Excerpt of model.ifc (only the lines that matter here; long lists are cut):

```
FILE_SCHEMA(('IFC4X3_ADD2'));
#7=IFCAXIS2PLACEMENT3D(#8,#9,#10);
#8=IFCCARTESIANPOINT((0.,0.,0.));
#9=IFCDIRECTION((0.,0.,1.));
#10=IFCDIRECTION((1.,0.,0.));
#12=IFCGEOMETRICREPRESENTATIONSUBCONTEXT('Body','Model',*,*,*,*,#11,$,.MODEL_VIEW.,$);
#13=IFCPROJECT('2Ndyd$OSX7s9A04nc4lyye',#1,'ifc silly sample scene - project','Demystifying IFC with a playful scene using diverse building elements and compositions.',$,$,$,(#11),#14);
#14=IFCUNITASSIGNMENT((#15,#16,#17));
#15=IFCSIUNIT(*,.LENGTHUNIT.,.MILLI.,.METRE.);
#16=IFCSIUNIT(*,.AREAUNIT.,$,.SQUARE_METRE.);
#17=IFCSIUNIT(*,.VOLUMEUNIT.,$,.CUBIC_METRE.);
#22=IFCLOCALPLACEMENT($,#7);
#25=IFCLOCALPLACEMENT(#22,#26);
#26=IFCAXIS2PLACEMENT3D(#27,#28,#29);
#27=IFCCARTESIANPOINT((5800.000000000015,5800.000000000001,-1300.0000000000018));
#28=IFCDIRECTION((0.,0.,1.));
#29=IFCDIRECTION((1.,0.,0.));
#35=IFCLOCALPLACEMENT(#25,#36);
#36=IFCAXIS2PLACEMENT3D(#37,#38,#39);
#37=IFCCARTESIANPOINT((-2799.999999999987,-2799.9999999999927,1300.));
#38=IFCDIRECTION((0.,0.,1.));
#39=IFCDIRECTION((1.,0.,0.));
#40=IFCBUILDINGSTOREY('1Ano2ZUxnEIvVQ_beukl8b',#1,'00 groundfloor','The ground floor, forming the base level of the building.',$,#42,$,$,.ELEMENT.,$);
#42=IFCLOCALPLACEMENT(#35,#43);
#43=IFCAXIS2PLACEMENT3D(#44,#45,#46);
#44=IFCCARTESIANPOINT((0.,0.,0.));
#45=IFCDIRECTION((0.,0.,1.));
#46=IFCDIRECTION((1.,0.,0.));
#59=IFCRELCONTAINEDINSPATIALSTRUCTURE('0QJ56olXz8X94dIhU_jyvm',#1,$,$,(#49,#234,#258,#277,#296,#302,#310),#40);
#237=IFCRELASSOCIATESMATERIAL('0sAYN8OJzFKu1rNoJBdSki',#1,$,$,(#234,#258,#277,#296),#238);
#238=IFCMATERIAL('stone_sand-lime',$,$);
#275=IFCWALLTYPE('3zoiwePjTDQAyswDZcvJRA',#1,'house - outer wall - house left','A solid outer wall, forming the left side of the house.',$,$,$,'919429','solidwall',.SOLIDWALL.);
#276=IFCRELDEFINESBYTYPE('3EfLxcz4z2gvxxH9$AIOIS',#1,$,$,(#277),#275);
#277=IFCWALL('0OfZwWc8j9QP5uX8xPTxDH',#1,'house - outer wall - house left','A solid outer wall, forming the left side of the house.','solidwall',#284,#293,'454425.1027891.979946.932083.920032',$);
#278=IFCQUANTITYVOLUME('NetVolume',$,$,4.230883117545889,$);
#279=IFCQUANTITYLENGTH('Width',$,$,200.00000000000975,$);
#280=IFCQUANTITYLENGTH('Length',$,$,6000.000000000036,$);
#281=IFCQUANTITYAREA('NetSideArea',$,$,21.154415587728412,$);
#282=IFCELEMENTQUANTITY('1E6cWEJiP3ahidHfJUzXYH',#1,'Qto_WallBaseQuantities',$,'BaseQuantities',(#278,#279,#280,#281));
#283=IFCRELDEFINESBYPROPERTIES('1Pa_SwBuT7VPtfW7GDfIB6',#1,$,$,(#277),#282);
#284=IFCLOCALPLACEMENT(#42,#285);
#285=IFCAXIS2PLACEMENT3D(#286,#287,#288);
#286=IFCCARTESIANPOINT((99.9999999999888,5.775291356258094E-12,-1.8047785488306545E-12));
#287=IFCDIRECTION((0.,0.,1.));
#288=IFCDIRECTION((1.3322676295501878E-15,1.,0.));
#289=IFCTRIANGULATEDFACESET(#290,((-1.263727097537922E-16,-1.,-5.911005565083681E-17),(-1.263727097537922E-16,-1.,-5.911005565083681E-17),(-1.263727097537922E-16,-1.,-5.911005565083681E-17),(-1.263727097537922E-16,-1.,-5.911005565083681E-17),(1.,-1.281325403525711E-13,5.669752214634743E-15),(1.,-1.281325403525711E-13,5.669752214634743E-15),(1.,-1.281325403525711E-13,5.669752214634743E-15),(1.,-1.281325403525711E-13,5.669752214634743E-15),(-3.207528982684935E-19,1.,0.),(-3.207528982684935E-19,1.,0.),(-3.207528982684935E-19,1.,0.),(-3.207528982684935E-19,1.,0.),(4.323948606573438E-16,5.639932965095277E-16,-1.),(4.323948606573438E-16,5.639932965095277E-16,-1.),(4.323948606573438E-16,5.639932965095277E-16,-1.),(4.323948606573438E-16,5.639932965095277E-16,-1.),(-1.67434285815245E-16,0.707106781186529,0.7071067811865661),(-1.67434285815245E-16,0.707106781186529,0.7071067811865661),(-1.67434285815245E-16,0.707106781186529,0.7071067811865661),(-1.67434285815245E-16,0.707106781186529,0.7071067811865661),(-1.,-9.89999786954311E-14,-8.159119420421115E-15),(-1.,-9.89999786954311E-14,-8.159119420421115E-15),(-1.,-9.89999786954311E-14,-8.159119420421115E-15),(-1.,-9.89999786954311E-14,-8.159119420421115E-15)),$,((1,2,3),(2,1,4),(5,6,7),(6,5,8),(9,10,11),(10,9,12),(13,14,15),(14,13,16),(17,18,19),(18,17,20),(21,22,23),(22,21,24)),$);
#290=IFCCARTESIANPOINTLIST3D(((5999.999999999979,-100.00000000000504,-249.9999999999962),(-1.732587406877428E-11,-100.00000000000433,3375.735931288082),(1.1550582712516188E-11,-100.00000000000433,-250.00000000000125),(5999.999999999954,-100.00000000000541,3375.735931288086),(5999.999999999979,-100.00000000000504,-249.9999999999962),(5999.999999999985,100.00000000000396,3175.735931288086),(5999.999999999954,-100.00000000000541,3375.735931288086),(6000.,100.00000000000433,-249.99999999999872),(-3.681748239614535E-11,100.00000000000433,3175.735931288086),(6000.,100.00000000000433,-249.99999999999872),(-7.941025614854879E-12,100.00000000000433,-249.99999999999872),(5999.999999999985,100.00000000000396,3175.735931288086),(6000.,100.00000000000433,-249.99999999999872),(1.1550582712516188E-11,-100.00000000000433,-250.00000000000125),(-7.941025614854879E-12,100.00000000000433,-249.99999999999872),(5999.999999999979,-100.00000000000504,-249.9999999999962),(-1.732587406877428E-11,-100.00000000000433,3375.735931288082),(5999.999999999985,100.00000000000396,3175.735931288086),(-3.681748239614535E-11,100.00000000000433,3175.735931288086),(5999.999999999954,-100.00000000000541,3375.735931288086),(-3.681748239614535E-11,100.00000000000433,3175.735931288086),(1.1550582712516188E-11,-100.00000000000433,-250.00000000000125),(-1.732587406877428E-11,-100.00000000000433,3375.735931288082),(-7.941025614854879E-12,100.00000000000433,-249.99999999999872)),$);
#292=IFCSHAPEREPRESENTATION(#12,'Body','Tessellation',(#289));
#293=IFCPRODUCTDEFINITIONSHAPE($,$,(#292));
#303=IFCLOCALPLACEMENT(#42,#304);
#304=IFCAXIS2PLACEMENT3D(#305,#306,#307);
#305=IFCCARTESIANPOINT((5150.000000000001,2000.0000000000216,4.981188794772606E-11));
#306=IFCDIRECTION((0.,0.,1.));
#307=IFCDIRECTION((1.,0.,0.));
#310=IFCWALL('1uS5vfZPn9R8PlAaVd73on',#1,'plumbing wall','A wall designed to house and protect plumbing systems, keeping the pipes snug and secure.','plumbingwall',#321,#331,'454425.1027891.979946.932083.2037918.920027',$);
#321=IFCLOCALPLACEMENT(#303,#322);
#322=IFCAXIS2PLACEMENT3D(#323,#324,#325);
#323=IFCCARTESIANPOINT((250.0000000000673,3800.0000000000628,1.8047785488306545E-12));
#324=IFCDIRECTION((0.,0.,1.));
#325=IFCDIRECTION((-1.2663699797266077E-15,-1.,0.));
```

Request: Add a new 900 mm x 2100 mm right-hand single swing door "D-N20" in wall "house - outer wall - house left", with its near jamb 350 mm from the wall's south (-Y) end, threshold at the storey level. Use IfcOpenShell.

```python
import numpy as np
import ifcopenshell
import ifcopenshell.api.feature
import ifcopenshell.api.geometry
import ifcopenshell.api.pset
import ifcopenshell.api.root
import ifcopenshell.api.spatial
import ifcopenshell.geom
import ifcopenshell.util.element
import ifcopenshell.util.placement
import ifcopenshell.util.representation
import ifcopenshell.util.shape
import ifcopenshell.util.unit

model = ifcopenshell.open("model.ifc")
unit_scale = ifcopenshell.util.unit.calculate_unit_scale(model)
area_scale = ifcopenshell.util.unit.calculate_unit_scale(model, "AREAUNIT")
volume_scale = ifcopenshell.util.unit.calculate_unit_scale(model, "VOLUMEUNIT")
settings = ifcopenshell.geom.settings()


def volume(element):
    """Net volume in cubic metres, openings subtracted."""
    shape = ifcopenshell.geom.create_shape(settings, element)
    return ifcopenshell.util.shape.get_volume(shape.geometry)


wall = model.by_guid("0OfZwWc8j9QP5uX8xPTxDH")
storey = ifcopenshell.util.element.get_container(wall, ifc_class="IfcBuildingStorey")
context = ifcopenshell.util.representation.get_context(model, "Model", "Body", "MODEL_VIEW")
before = volume(wall)

width, height, from_end, sill = 0.9, 2.1, 0.35, 0.0  # metres

# The wall runs along its own X axis, and the end named is its -X end.
wall_shape = ifcopenshell.geom.create_shape(settings, wall)
x, y, z = ifcopenshell.util.shape.get_vertices(wall_shape.geometry).T
start = x.min() + from_end
face, thickness = float(y.min()), float(y.max() - y.min())
wall_matrix = ifcopenshell.util.placement.get_local_placement(wall.ObjectPlacement)
level = ifcopenshell.util.placement.get_local_placement(storey.ObjectPlacement)[2, 3]


def in_wall(x, y):
    """Placement at x, y metres in the wall's axes, at sill height."""
    matrix = wall_matrix.copy()
    matrix[:, 3] = wall_matrix @ np.array([x / unit_scale, y / unit_scale, 0.0, 1.0])
    matrix[2, 3] = level + sill / unit_scale
    return matrix


# Opening: a box that overshoots both wall faces by 50 mm.
opening = ifcopenshell.api.root.create_entity(model, ifc_class="IfcOpeningElement", predefined_type="OPENING")
box = ifcopenshell.api.geometry.add_wall_representation(
    model, context=context, length=width, height=height, thickness=thickness + 0.1
)
ifcopenshell.api.geometry.assign_representation(model, product=opening, representation=box)
ifcopenshell.api.geometry.edit_object_placement(model, product=opening, matrix=in_wall(start, face - 0.05), is_si=False)
ifcopenshell.api.feature.add_feature(model, feature=opening, element=wall)

door = ifcopenshell.api.root.create_entity(model, ifc_class="IfcDoor", name="D-N20", predefined_type="DOOR")
door.OverallWidth, door.OverallHeight = width / unit_scale, height / unit_scale
door.OperationType = "SINGLE_SWING_RIGHT"
body = ifcopenshell.api.geometry.add_door_representation(
    model,
    context=context,
    overall_width=door.OverallWidth,
    overall_height=door.OverallHeight,
    operation_type="SINGLE_SWING_RIGHT",
    lining_properties={"LiningDepth": thickness / unit_scale, "ThresholdDepth": thickness / unit_scale},
)
ifcopenshell.api.geometry.assign_representation(model, product=door, representation=body)
ifcopenshell.api.spatial.assign_container(model, products=[door], relating_structure=storey)
ifcopenshell.api.feature.add_filling(model, opening=opening, element=door)

# The lining spans the wall, so the door starts at the wall face.
ifcopenshell.api.geometry.edit_object_placement(model, product=door, matrix=in_wall(start, face), is_si=False)

after = volume(wall)

# Update the wall's stored quantities.
qto = model.by_id(ifcopenshell.util.element.get_pset(wall, "Qto_WallBaseQuantities", should_inherit=False)["id"])
ifcopenshell.api.pset.edit_qto(model, qto=qto, properties={
    "NetVolume": after / volume_scale,
    "NetSideArea": after / thickness / area_scale,
})

print(f"wall volume {before:.3f} -> {after:.3f} m3")

model.write("model_rev.ifc")
```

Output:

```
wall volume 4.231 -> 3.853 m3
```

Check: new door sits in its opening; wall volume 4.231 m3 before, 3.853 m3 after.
